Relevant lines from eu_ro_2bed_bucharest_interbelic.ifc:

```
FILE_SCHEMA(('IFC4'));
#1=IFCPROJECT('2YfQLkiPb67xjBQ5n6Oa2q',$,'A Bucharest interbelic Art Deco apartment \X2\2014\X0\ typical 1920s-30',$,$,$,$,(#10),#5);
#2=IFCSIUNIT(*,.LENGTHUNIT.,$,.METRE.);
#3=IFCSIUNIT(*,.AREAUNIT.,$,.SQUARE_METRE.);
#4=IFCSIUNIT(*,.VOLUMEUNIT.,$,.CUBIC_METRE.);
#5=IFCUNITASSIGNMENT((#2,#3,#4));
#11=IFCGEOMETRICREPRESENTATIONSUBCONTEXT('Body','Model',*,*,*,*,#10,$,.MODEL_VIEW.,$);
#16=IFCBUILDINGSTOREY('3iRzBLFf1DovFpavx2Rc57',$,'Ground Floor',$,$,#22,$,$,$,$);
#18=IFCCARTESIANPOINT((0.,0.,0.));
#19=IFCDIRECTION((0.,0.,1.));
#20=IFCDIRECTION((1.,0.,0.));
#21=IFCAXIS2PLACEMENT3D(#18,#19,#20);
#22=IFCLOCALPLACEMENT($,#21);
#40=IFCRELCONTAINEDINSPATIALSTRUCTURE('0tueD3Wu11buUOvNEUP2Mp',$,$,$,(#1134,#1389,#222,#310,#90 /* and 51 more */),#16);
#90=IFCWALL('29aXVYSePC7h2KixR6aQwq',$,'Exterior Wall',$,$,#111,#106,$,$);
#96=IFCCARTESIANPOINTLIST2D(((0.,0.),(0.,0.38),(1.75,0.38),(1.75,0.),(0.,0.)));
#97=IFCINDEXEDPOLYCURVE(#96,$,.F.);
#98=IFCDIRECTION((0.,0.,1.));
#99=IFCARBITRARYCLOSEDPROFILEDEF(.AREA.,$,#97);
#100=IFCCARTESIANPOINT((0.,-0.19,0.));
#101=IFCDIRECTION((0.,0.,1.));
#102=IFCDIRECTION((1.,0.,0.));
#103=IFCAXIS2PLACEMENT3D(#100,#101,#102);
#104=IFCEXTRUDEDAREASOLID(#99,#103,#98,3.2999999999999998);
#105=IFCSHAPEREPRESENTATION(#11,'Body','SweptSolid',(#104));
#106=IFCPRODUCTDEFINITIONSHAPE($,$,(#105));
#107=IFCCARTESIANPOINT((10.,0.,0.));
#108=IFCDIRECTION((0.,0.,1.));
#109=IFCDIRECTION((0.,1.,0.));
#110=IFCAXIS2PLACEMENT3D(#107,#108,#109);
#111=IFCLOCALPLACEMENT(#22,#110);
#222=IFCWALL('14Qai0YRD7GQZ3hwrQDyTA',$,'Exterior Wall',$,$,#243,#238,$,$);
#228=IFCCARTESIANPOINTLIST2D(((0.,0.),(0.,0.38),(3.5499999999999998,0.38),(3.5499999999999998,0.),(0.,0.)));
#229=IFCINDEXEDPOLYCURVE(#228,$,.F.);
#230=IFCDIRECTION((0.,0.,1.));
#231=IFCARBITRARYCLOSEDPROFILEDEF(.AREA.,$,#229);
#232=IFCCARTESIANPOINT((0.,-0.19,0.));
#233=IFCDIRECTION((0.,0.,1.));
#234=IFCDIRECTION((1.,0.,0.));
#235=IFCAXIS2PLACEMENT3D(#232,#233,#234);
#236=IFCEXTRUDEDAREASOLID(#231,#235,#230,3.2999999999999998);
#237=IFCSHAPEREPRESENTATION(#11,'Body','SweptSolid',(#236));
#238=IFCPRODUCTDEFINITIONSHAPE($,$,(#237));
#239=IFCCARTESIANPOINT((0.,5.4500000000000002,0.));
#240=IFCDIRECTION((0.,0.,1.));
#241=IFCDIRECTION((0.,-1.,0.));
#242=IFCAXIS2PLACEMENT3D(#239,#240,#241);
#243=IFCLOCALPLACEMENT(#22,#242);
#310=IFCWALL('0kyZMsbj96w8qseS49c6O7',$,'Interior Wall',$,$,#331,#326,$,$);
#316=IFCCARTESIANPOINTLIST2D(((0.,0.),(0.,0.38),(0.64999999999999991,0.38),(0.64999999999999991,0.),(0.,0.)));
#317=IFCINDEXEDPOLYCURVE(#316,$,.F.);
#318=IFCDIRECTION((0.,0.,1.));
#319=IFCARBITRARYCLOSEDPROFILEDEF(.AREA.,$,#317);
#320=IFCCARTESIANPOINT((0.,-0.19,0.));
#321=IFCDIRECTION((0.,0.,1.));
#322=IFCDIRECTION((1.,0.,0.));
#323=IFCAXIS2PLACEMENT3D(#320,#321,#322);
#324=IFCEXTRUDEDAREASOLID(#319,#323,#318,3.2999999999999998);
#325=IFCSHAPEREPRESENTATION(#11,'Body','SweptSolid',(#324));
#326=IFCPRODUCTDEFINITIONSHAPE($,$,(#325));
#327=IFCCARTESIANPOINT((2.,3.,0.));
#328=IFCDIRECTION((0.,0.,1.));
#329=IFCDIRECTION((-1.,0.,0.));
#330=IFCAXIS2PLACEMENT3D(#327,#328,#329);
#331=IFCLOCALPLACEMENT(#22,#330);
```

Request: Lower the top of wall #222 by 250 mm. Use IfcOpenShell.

```python
import ifcopenshell
import ifcopenshell.geom
import ifcopenshell.util.representation
import ifcopenshell.util.shape

model = ifcopenshell.open("eu_ro_2bed_bucharest_interbelic.ifc")
settings = ifcopenshell.geom.settings()


def volume(element):
    """Net volume in cubic metres, openings subtracted."""
    shape = ifcopenshell.geom.create_shape(settings, element)
    return ifcopenshell.util.shape.get_volume(shape.geometry)


wall = model.by_guid("14Qai0YRD7GQZ3hwrQDyTA")
before = volume(wall)

body = ifcopenshell.util.representation.get_representation(wall, "Model", "Body")
solid = body.Items[0]
old_height = solid.Depth
solid.Depth -= 0.25
after = volume(wall)

print(f"height {old_height:g} -> {solid.Depth:g}, volume {before:.3f} -> {after:.3f} m3")

model.write("eu_ro_2bed_bucharest_interbelic_updated.ifc")
```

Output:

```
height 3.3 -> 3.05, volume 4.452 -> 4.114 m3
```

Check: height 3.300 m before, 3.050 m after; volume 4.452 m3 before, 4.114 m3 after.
